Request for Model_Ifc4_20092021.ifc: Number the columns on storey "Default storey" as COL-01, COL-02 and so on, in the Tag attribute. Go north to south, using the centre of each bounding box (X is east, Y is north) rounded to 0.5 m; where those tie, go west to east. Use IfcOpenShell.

First a look at what the model holds.

```python
import ifcopenshell
import ifcopenshell.util.element
import ifcopenshell.util.placement

model = ifcopenshell.open("Model_Ifc4_20092021.ifc")
print(model.schema)
storey = next(s for s in model.by_type("IfcBuildingStorey") if s.Name == "Default storey")
columns = [e for e in ifcopenshell.util.element.get_decomposition(storey) if e.is_a("IfcColumn")]
for e in sorted(columns, key=lambda e: e.id()):
    origin = ifcopenshell.util.placement.get_local_placement(e.ObjectPlacement)[:3, 3]
    print(e.id(), e.Tag, e.Name, origin.round(2) + 0.0, sep=" | ")
```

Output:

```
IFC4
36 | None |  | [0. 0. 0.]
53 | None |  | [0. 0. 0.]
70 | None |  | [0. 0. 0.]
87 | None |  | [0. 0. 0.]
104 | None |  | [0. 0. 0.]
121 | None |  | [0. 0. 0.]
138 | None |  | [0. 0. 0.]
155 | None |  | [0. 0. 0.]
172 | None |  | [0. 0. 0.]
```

```python
import ifcopenshell
import ifcopenshell.geom
import ifcopenshell.util.element
import ifcopenshell.util.shape

model = ifcopenshell.open("Model_Ifc4_20092021.ifc")
settings = ifcopenshell.geom.settings()
settings.set("use-world-coords", True)


def centre(element):
    shape = ifcopenshell.geom.create_shape(settings, element)
    return ifcopenshell.util.shape.get_bbox_centroid(shape.geometry)


storey = next(s for s in model.by_type("IfcBuildingStorey") if s.Name == "Default storey")
columns = [e for e in ifcopenshell.util.element.get_decomposition(storey) if e.is_a("IfcColumn")]

# Insertion points can sit at a corner or the storey origin, so sort by the geometry (in metres).
centres = {e: centre(e) for e in columns}
columns.sort(key=lambda e: (-round(centres[e][1] / 0.5), centres[e][0]))

for i, e in enumerate(columns, start=1):
    number = f"COL-{i:02d}"
    e.Tag = number
    print(e.id(), number)

model.write("Model_Ifc4_20092021_updated.ifc")
```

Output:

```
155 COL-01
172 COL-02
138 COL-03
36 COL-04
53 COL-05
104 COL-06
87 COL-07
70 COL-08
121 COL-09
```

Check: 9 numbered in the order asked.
